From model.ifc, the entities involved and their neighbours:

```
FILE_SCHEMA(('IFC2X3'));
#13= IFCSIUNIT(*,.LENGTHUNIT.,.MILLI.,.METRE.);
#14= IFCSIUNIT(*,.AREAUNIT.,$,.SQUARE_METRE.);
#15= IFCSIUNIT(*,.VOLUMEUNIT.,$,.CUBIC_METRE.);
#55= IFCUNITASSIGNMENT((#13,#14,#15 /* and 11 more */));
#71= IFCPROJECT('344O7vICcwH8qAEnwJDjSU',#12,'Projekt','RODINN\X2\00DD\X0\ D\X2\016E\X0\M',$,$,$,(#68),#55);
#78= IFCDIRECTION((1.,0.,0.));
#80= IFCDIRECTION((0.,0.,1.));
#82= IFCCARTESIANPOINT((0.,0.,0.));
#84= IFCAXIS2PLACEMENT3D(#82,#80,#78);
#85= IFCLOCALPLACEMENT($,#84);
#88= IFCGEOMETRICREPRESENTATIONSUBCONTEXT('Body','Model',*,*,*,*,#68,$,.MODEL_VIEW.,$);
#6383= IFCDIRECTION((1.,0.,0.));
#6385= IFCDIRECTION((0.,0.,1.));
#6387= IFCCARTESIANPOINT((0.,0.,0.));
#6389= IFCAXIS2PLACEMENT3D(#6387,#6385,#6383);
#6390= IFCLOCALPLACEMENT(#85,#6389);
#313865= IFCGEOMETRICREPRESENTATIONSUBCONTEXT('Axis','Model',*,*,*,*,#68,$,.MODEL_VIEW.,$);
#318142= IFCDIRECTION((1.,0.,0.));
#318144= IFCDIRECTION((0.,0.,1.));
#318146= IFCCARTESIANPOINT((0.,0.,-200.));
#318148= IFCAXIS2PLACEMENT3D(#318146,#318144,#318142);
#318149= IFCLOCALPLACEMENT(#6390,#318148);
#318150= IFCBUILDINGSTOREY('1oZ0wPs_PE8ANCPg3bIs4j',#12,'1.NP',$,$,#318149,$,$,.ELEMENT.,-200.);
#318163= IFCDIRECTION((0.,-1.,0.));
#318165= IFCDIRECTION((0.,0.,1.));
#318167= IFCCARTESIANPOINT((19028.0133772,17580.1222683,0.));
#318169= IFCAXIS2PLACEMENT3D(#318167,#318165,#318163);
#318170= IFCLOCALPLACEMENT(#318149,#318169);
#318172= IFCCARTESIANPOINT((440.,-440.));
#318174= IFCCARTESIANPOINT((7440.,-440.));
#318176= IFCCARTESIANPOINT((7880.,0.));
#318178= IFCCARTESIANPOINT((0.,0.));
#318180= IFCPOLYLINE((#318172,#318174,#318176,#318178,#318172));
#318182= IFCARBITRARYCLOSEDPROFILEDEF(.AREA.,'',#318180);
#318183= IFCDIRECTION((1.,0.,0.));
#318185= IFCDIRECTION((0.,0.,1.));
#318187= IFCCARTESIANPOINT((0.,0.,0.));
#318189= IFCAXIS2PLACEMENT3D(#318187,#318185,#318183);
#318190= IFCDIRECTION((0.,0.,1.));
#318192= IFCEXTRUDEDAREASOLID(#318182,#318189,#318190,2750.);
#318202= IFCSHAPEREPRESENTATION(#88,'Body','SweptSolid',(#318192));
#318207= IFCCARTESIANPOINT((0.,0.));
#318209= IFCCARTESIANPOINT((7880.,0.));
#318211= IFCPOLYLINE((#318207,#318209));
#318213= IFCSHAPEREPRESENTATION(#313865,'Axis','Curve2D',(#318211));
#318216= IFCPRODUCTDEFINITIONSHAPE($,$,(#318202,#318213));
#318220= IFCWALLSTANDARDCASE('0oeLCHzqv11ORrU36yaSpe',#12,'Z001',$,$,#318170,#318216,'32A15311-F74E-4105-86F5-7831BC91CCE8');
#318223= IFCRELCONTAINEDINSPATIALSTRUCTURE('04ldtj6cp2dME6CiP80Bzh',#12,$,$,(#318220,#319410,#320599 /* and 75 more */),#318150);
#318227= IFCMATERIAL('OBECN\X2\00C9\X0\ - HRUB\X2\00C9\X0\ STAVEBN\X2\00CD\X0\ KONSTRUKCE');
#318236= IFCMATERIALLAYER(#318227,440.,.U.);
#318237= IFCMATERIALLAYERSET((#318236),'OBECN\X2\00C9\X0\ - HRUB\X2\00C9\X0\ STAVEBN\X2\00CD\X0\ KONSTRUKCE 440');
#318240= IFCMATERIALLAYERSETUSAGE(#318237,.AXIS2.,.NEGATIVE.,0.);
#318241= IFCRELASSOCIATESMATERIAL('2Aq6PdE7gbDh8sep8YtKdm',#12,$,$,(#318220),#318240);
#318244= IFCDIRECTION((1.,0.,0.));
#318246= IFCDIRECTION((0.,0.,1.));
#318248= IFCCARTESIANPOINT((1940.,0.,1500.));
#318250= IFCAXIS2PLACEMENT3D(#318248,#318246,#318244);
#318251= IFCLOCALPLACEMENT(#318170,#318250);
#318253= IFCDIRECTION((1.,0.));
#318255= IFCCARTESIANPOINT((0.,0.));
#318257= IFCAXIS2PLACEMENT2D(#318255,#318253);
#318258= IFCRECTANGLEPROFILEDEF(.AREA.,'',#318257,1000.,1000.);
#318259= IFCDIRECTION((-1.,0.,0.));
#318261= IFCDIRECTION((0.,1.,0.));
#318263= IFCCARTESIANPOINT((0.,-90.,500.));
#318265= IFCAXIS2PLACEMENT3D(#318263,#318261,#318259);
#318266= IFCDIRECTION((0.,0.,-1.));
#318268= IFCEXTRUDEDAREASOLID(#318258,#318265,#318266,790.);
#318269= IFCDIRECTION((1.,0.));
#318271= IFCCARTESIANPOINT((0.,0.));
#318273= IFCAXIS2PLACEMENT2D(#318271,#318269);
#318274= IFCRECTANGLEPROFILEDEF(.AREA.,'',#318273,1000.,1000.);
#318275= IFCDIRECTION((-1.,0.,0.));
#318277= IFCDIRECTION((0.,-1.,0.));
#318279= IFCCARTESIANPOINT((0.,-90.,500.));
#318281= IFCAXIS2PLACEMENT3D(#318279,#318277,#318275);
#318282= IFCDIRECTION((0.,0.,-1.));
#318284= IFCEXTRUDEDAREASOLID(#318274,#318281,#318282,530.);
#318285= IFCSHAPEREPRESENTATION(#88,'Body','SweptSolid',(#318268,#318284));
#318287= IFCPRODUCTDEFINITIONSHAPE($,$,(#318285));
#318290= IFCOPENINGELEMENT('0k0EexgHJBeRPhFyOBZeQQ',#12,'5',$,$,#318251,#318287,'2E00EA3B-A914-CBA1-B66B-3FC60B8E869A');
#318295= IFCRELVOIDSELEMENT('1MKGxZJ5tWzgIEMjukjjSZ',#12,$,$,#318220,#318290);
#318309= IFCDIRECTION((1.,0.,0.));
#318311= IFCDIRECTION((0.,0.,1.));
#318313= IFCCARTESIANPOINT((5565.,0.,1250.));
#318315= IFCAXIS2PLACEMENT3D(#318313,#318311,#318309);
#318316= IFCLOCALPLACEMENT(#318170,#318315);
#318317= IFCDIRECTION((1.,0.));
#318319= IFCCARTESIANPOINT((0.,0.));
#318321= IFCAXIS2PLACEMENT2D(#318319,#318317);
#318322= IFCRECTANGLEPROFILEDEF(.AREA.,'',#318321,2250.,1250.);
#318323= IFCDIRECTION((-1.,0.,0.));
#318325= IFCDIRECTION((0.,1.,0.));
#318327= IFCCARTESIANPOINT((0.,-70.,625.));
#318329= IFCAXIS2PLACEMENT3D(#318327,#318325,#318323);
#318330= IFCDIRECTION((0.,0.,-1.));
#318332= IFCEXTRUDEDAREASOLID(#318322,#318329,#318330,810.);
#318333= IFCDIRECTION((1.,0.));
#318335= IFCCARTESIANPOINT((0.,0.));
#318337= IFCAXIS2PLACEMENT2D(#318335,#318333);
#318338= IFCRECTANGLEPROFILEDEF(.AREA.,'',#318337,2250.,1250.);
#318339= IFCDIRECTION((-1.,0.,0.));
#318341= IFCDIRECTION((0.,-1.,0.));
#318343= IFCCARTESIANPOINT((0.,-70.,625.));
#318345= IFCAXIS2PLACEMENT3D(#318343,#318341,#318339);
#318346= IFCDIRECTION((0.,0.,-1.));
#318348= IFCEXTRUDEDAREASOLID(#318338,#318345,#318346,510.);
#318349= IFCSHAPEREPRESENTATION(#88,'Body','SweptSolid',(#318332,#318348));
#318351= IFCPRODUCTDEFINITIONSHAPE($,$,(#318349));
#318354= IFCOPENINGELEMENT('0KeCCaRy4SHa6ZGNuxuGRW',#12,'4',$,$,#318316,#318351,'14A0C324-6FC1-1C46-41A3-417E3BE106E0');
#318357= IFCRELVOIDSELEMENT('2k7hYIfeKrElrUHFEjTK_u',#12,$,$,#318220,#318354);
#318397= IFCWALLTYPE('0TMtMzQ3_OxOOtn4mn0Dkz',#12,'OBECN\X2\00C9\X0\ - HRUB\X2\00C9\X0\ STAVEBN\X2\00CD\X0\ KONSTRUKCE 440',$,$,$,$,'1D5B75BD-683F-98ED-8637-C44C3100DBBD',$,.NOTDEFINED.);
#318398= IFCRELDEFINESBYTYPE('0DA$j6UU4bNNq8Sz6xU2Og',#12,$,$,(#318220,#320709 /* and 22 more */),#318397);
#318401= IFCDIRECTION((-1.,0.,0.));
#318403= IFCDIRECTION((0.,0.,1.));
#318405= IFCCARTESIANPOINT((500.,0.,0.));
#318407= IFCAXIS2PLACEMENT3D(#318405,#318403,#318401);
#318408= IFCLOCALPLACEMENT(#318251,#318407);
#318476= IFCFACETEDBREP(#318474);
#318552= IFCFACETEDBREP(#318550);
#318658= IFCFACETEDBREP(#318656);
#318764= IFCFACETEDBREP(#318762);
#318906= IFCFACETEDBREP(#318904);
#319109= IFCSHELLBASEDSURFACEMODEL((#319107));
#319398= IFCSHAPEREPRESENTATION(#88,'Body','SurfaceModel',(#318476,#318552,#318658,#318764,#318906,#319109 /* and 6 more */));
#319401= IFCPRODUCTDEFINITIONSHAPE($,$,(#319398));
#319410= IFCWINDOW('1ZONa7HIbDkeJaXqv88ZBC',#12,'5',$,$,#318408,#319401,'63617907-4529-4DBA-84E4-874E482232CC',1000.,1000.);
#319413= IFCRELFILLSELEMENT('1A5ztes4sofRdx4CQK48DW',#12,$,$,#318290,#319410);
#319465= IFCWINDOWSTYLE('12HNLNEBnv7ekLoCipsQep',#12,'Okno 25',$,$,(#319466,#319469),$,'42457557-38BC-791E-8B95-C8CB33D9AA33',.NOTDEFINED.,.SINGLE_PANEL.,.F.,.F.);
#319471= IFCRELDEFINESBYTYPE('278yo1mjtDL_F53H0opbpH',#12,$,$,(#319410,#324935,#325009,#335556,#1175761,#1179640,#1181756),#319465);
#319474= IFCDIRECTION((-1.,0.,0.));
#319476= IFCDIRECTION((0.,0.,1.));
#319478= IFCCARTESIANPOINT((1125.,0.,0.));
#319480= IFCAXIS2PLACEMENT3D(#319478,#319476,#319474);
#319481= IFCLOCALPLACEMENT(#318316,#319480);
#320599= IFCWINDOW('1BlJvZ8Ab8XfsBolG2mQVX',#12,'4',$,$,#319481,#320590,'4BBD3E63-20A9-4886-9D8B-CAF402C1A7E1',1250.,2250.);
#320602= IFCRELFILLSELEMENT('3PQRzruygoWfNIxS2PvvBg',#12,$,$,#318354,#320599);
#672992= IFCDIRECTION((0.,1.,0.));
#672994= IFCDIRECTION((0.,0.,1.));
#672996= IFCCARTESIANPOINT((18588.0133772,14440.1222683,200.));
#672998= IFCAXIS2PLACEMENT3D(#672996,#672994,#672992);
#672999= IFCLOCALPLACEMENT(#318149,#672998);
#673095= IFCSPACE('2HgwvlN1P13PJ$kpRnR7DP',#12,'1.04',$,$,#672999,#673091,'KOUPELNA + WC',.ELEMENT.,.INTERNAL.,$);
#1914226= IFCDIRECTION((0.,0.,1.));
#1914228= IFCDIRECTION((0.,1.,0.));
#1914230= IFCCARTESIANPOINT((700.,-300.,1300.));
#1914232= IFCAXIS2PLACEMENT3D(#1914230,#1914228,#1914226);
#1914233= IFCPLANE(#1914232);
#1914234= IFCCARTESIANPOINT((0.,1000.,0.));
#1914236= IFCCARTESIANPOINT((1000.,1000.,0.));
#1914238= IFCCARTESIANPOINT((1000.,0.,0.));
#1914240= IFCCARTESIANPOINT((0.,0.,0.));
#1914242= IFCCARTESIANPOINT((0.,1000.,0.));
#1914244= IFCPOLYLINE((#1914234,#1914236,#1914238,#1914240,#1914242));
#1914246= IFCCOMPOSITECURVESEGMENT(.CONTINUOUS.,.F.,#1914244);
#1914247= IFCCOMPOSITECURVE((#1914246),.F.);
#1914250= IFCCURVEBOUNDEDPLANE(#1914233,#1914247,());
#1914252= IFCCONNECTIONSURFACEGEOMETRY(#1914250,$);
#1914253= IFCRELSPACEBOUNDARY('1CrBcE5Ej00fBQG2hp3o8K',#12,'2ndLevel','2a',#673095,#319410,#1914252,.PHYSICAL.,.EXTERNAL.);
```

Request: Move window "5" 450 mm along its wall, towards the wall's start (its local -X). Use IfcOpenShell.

```python
import numpy as np
import ifcopenshell
import ifcopenshell.api.geometry
import ifcopenshell.util.placement
import ifcopenshell.util.unit

model = ifcopenshell.open("model.ifc")
unit_scale = ifcopenshell.util.unit.calculate_unit_scale(model)

window = model.by_id(319410)
opening = window.FillsVoids[0].RelatingOpeningElement
wall = opening.VoidsElements[0].RelatingBuildingElement

wall_matrix = ifcopenshell.util.placement.get_local_placement(wall.ObjectPlacement)
shift = wall_matrix[:3, 0] * -0.45 / unit_scale
before = ifcopenshell.util.placement.get_local_placement(window.ObjectPlacement)[:3, 3].copy()

# The window is placed relative to its opening, so it follows when the opening moves.
matrix = ifcopenshell.util.placement.get_local_placement(opening.ObjectPlacement)
matrix[:3, 3] += shift
ifcopenshell.api.geometry.edit_object_placement(
    model, product=opening, matrix=matrix, is_si=False, should_transform_children=True
)

# Space boundary surfaces are stored in each space's coordinates; move them too.
for rel in window.ProvidesBoundaries:
    if not rel.ConnectionGeometry:
        continue
    surface = rel.ConnectionGeometry.SurfaceOnRelatingElement.BasisSurface
    space_matrix = ifcopenshell.util.placement.get_local_placement(rel.RelatingSpace.ObjectPlacement)
    point = np.array(surface.Position.Location.Coordinates) + space_matrix[:3, :3].T @ shift
    surface.Position = model.createIfcAxis2Placement3D(
        model.createIfcCartesianPoint(point.tolist()), surface.Position.Axis, surface.Position.RefDirection
    )

after = ifcopenshell.util.placement.get_local_placement(window.ObjectPlacement)[:3, 3]
print("window moved by", (after - before).round(3) + 0.0)

model.write("model-out.ifc")
```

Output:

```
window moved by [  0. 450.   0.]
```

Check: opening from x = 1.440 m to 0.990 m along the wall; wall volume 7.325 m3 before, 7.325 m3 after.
